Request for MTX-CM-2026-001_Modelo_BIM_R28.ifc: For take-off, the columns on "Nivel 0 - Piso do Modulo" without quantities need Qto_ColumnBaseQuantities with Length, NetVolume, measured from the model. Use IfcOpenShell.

First a look at what the model holds.

```python
import ifcopenshell
import ifcopenshell.util.element
import ifcopenshell.util.unit

model = ifcopenshell.open("MTX-CM-2026-001_Modelo_BIM_R28.ifc")
print(model.schema)
for unit_type in ("LENGTHUNIT", "AREAUNIT", "VOLUMEUNIT"):
    print(unit_type, ifcopenshell.util.unit.calculate_unit_scale(model, unit_type))
storey = next(s for s in model.by_type("IfcBuildingStorey") if s.Name == "Nivel 0 - Piso do Modulo")
columns = [e for e in ifcopenshell.util.element.get_decomposition(storey) if e.is_a("IfcColumn")]
for e in sorted(columns, key=lambda e: e.id()):
    print(e.id(), e.is_a(), e.Name, list(ifcopenshell.util.element.get_psets(e, qtos_only=True)), sep=" | ")
```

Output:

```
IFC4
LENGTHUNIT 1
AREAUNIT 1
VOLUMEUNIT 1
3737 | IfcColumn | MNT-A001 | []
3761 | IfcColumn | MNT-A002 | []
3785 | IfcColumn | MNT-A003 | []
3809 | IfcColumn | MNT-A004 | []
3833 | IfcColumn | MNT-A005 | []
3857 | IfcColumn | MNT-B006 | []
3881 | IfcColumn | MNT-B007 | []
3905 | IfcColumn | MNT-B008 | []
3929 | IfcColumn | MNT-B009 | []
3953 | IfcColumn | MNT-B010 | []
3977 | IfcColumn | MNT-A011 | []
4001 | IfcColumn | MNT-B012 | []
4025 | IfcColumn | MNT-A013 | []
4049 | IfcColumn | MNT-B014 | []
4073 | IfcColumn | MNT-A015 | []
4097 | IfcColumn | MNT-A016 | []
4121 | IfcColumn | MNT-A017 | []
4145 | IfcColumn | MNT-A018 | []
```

```python
import ifcopenshell
import ifcopenshell.api.pset
import ifcopenshell.geom
import ifcopenshell.util.element
import ifcopenshell.util.shape
import ifcopenshell.util.unit

model = ifcopenshell.open("MTX-CM-2026-001_Modelo_BIM_R28.ifc")
unit_scale = ifcopenshell.util.unit.calculate_unit_scale(model)
volume_scale = ifcopenshell.util.unit.calculate_unit_scale(model, "VOLUMEUNIT")
settings = ifcopenshell.geom.settings()

storey = next(s for s in model.by_type("IfcBuildingStorey") if s.Name == "Nivel 0 - Piso do Modulo")
columns = [e for e in ifcopenshell.util.element.get_decomposition(storey) if e.is_a("IfcColumn")]

for e in sorted(columns, key=lambda e: e.id()):
    if ifcopenshell.util.element.get_psets(e, qtos_only=True, should_inherit=False):
        continue
    # Geometry comes back in metres, in the element's own axes.
    shape = ifcopenshell.geom.create_shape(settings, e)
    values = {
        "Length": ifcopenshell.util.shape.get_z(shape.geometry) / unit_scale,
        "NetVolume": ifcopenshell.util.shape.get_volume(shape.geometry) / volume_scale,
    }
    qto = ifcopenshell.api.pset.add_qto(model, product=e, name="Qto_ColumnBaseQuantities")
    ifcopenshell.api.pset.edit_qto(model, qto=qto, properties=values)
    print(e.id(), {k: round(v, 3) for k, v in values.items()})

model.write("MTX-CM-2026-001_Modelo_BIM_R28_rev.ifc")
```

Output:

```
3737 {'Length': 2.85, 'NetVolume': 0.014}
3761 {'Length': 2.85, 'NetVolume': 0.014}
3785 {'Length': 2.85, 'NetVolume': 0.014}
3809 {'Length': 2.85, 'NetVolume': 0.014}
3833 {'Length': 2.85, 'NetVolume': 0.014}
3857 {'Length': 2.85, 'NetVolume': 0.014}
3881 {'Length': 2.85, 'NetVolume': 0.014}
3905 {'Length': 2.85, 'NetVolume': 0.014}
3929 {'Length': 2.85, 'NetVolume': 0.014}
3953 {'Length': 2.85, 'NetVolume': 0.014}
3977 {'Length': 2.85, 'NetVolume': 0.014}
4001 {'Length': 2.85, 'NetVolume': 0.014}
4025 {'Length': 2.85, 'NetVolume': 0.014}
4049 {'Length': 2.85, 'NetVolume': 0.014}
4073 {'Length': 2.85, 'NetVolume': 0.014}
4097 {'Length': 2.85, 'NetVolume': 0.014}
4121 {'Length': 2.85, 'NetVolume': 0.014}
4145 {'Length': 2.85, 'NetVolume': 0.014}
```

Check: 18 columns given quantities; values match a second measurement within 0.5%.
